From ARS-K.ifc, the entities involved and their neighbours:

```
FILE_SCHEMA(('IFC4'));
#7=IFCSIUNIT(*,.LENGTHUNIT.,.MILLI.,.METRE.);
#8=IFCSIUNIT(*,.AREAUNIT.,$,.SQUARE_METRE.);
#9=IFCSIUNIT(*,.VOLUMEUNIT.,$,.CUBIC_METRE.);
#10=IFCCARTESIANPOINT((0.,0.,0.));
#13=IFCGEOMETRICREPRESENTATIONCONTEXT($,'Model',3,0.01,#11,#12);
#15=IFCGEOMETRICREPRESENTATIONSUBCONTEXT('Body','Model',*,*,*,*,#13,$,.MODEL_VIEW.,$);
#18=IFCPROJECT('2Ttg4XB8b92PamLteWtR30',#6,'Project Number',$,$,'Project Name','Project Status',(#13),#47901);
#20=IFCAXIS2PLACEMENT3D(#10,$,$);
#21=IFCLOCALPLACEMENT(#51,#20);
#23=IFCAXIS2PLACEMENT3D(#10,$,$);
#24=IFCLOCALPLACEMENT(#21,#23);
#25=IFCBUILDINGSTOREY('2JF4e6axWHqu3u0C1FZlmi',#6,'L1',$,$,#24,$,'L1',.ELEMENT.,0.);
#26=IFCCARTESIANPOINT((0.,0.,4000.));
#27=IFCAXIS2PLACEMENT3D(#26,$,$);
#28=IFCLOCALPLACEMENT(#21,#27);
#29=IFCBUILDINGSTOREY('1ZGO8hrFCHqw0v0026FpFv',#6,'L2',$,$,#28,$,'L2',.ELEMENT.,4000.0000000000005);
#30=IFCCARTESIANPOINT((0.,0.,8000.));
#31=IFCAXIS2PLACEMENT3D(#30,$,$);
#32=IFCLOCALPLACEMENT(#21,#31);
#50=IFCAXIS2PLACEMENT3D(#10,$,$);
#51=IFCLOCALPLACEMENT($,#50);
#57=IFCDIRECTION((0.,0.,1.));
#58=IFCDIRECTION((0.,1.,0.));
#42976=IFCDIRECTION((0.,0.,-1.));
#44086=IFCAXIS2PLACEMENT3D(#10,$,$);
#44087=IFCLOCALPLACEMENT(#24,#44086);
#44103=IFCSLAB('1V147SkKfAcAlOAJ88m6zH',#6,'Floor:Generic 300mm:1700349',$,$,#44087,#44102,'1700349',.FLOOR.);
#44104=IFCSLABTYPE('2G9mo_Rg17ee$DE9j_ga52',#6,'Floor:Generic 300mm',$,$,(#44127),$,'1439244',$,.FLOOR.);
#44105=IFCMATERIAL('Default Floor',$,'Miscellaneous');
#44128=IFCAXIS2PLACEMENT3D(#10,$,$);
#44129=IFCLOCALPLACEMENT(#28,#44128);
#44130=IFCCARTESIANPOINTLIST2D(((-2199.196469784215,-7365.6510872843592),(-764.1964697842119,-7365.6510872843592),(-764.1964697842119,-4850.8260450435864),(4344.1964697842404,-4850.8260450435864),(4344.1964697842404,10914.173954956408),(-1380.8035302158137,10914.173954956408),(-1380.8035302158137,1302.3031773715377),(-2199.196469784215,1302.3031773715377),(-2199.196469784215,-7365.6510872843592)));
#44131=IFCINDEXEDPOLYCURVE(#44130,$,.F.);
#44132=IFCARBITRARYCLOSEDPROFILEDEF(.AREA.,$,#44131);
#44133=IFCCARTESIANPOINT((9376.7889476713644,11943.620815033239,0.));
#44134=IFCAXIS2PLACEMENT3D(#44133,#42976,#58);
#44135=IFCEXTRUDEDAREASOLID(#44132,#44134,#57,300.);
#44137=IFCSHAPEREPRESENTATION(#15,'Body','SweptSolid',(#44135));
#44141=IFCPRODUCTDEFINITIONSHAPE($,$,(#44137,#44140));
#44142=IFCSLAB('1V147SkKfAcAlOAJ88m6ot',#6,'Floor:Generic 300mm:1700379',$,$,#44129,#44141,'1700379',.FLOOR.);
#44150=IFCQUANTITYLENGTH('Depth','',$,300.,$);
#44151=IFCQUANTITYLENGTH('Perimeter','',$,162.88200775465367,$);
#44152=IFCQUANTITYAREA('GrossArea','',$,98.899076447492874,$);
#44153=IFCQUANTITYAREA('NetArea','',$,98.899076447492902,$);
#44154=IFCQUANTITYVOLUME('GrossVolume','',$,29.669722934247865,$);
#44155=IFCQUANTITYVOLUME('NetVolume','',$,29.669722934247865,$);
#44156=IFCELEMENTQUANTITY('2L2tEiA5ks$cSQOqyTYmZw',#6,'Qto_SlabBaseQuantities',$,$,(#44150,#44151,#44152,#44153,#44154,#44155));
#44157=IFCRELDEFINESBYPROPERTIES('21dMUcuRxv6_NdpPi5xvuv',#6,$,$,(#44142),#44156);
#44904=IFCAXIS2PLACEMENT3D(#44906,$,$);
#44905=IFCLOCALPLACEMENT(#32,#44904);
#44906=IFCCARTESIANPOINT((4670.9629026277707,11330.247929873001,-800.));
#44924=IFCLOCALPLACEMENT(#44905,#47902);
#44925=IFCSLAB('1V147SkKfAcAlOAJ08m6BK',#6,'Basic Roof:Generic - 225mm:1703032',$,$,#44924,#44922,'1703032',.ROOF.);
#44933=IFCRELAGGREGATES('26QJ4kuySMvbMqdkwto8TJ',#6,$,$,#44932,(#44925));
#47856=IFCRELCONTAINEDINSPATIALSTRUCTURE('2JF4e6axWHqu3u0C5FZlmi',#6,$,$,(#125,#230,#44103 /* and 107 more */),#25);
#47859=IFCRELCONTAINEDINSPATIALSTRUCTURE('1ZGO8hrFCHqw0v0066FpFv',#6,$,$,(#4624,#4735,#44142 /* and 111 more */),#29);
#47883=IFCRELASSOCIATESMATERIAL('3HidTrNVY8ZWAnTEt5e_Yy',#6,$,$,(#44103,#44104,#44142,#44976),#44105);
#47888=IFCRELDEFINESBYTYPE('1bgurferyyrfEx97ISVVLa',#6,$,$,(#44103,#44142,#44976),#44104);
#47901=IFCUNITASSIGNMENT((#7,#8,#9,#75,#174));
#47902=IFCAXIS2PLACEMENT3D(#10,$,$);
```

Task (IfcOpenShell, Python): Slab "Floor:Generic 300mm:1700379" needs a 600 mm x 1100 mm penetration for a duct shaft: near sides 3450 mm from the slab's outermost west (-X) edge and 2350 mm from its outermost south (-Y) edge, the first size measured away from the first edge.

```python
import numpy as np
import ifcopenshell
import ifcopenshell.api.feature
import ifcopenshell.api.geometry
import ifcopenshell.api.pset
import ifcopenshell.api.root
import ifcopenshell.geom
import ifcopenshell.util.element
import ifcopenshell.util.placement
import ifcopenshell.util.representation
import ifcopenshell.util.shape
import ifcopenshell.util.unit

model = ifcopenshell.open("ARS-K.ifc")
unit_scale = ifcopenshell.util.unit.calculate_unit_scale(model)
area_scale = ifcopenshell.util.unit.calculate_unit_scale(model, "AREAUNIT")
volume_scale = ifcopenshell.util.unit.calculate_unit_scale(model, "VOLUMEUNIT")
settings = ifcopenshell.geom.settings()


def volume(element):
    """Net volume in cubic metres, openings subtracted."""
    shape = ifcopenshell.geom.create_shape(settings, element)
    return ifcopenshell.util.shape.get_volume(shape.geometry)


slab = model.by_guid("1V147SkKfAcAlOAJ88m6ot")
before = volume(slab)

# Extent in the slab's own axes, in metres. The edges named are its -X and -Y sides.
slab_shape = ifcopenshell.geom.create_shape(settings, slab)
vertices = ifcopenshell.util.shape.get_vertices(slab_shape.geometry)
x_min, y_min, bottom = vertices.min(axis=0)
top = vertices[:, 2].max()

opening = ifcopenshell.api.root.create_entity(model, ifc_class="IfcOpeningElement", name="Duct shaft opening", predefined_type="OPENING")
context = ifcopenshell.util.representation.get_context(model, "Model", "Body", "MODEL_VIEW")
width, depth = 0.6, 1.1
outline = [(0.0, 0.0), (width, 0.0), (width, depth), (0.0, depth), (0.0, 0.0)]
# Overshoot both faces by 50 mm so the cut is clean.
shape = ifcopenshell.api.geometry.add_slab_representation(
    model, context=context, depth=top - bottom + 0.1, polyline=outline
)
ifcopenshell.api.geometry.assign_representation(model, product=opening, representation=shape)

matrix = ifcopenshell.util.placement.get_local_placement(slab.ObjectPlacement)
matrix[:, 3] = matrix @ np.append(np.array([x_min + 3.45, y_min + 2.35, bottom - 0.05]) / unit_scale, 1.0)
ifcopenshell.api.geometry.edit_object_placement(model, product=opening, matrix=matrix, is_si=False)
ifcopenshell.api.feature.add_feature(model, feature=opening, element=slab)

after = volume(slab)

# Update the slab's stored quantities.
qto = model.by_id(ifcopenshell.util.element.get_pset(slab, "Qto_SlabBaseQuantities", should_inherit=False)["id"])
ifcopenshell.api.pset.edit_qto(model, qto=qto, properties={
    "NetArea": after / (top - bottom) / area_scale,
    "NetVolume": after / volume_scale,
})

print(f"slab volume {before:.3f} -> {after:.3f} m3")

model.write("ARS-K_edited.ifc")
```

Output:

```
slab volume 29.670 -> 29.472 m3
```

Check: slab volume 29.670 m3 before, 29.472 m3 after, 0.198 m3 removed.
